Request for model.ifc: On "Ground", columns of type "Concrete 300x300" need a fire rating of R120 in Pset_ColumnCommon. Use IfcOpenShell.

First a look at what the model holds.

```python
import ifcopenshell
import ifcopenshell.util.element

model = ifcopenshell.open("model.ifc")
print(model.schema)
storey = next(s for s in model.by_type("IfcBuildingStorey") if s.Name == "Ground")
columns = [e for e in ifcopenshell.util.element.get_decomposition(storey) if e.is_a("IfcColumn")]
seen = {}
for e in columns:
    element_type = ifcopenshell.util.element.get_type(e)
    key = (element_type.Name if element_type != e and element_type else None, ifcopenshell.util.element.get_pset(e, "Pset_ColumnCommon", "FireRating"))
    seen[key] = seen.get(key, 0) + 1
for (name, value), count in sorted(seen.items(), key=str):
    print(count, "x", name, "|", value)
```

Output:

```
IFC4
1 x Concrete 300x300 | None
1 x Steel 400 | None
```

```python
import ifcopenshell
import ifcopenshell.api.pset
import ifcopenshell.util.element

model = ifcopenshell.open("model.ifc")

storey = next(s for s in model.by_type("IfcBuildingStorey") if s.Name == "Ground")
columns = [e for e in ifcopenshell.util.element.get_decomposition(storey) if e.is_a("IfcColumn")]

count = 0
for e in columns:
    element_type = ifcopenshell.util.element.get_type(e)
    if element_type in (None, e) or element_type.Name != "Concrete 300x300":
        continue
    # add_pset returns the element's existing set when there is one.
    pset = ifcopenshell.api.pset.add_pset(model, product=e, name="Pset_ColumnCommon")
    ifcopenshell.api.pset.edit_pset(model, pset=pset, properties={"FireRating": "R120"})
    count += 1

print(count, "columns updated")

model.write("model-out.ifc")
```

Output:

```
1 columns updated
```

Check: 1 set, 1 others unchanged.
